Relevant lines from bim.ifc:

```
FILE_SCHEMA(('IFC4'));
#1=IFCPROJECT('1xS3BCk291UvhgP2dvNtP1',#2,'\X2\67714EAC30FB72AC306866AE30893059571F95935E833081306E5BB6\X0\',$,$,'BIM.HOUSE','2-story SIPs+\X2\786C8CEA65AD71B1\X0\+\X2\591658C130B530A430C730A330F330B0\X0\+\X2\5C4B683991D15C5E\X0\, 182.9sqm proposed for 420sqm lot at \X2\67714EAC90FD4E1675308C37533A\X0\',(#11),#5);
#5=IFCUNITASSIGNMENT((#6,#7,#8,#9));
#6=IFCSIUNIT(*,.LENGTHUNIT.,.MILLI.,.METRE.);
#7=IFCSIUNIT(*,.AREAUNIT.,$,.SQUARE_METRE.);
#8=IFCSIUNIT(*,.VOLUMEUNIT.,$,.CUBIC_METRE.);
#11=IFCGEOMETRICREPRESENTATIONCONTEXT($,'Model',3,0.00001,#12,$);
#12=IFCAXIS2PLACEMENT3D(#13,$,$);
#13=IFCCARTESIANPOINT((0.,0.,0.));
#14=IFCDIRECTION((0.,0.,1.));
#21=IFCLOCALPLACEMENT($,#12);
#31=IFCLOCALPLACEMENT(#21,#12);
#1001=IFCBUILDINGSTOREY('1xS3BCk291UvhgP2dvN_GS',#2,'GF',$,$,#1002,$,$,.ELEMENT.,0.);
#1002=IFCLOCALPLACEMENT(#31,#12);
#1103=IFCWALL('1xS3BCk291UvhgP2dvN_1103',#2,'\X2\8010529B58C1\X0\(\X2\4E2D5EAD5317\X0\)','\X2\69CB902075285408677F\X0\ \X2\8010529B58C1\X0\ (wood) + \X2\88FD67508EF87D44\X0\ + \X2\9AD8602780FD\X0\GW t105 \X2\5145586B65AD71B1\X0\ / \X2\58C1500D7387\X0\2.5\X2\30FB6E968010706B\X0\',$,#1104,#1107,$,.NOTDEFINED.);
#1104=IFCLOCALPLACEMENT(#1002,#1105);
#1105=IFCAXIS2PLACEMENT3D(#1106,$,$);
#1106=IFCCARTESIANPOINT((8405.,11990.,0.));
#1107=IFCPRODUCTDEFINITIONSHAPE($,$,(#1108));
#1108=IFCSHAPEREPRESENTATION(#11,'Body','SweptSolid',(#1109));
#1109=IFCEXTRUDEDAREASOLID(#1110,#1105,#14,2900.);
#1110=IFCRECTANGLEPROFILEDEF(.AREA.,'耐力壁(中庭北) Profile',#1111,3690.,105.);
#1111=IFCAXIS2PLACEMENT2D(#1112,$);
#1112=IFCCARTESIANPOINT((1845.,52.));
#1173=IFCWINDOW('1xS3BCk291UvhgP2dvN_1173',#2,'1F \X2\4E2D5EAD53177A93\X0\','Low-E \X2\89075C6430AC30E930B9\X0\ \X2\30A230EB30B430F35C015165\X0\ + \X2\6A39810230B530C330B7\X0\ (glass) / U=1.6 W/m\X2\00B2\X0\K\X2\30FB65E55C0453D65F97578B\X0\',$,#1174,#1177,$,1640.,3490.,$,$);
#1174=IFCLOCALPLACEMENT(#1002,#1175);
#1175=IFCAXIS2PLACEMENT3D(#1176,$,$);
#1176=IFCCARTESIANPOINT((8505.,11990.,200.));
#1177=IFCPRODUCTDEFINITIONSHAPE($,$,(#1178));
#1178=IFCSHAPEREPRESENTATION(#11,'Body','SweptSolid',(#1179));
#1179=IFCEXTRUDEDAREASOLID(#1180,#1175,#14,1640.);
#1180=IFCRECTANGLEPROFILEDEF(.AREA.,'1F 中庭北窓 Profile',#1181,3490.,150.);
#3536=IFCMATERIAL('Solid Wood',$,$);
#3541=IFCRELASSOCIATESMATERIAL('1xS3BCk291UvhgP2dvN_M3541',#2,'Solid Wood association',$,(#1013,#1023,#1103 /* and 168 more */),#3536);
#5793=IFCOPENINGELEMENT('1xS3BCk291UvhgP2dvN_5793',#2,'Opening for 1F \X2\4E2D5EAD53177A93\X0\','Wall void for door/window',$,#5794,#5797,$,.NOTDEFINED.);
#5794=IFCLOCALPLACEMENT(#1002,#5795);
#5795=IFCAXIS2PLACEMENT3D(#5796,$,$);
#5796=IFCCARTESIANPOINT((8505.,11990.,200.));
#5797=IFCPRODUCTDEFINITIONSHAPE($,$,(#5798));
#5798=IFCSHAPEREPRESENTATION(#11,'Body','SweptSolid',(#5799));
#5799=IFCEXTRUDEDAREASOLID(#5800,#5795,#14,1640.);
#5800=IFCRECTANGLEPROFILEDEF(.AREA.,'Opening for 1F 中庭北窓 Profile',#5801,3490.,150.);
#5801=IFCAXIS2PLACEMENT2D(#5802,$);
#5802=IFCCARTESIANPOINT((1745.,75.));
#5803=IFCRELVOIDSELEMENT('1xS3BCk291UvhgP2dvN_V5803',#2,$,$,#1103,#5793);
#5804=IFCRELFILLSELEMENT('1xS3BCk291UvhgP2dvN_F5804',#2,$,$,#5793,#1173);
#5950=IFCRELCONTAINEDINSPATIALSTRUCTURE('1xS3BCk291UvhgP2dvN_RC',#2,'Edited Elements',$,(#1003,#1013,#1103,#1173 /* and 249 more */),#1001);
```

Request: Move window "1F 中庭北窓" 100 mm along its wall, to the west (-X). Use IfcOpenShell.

```python
import ifcopenshell
import ifcopenshell.api.geometry
import ifcopenshell.util.placement
import ifcopenshell.util.unit

model = ifcopenshell.open("bim.ifc")
unit_scale = ifcopenshell.util.unit.calculate_unit_scale(model)

window = model.by_id(1173)
opening = window.FillsVoids[0].RelatingOpeningElement
wall = opening.VoidsElements[0].RelatingBuildingElement

wall_matrix = ifcopenshell.util.placement.get_local_placement(wall.ObjectPlacement)
shift = wall_matrix[:3, 0] * -0.1 / unit_scale
before = ifcopenshell.util.placement.get_local_placement(window.ObjectPlacement)[:3, 3].copy()

# The window is not placed relative to its opening, so move both.
for product in (opening, window):
    matrix = ifcopenshell.util.placement.get_local_placement(product.ObjectPlacement)
    matrix[:3, 3] += shift
    ifcopenshell.api.geometry.edit_object_placement(model, product=product, matrix=matrix, is_si=False)

after = ifcopenshell.util.placement.get_local_placement(window.ObjectPlacement)[:3, 3]
print("window moved by", (after - before).round(3) + 0.0)

model.write("bim_rev.ifc")
```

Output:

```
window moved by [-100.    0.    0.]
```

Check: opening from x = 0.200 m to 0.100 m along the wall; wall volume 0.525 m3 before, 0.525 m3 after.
